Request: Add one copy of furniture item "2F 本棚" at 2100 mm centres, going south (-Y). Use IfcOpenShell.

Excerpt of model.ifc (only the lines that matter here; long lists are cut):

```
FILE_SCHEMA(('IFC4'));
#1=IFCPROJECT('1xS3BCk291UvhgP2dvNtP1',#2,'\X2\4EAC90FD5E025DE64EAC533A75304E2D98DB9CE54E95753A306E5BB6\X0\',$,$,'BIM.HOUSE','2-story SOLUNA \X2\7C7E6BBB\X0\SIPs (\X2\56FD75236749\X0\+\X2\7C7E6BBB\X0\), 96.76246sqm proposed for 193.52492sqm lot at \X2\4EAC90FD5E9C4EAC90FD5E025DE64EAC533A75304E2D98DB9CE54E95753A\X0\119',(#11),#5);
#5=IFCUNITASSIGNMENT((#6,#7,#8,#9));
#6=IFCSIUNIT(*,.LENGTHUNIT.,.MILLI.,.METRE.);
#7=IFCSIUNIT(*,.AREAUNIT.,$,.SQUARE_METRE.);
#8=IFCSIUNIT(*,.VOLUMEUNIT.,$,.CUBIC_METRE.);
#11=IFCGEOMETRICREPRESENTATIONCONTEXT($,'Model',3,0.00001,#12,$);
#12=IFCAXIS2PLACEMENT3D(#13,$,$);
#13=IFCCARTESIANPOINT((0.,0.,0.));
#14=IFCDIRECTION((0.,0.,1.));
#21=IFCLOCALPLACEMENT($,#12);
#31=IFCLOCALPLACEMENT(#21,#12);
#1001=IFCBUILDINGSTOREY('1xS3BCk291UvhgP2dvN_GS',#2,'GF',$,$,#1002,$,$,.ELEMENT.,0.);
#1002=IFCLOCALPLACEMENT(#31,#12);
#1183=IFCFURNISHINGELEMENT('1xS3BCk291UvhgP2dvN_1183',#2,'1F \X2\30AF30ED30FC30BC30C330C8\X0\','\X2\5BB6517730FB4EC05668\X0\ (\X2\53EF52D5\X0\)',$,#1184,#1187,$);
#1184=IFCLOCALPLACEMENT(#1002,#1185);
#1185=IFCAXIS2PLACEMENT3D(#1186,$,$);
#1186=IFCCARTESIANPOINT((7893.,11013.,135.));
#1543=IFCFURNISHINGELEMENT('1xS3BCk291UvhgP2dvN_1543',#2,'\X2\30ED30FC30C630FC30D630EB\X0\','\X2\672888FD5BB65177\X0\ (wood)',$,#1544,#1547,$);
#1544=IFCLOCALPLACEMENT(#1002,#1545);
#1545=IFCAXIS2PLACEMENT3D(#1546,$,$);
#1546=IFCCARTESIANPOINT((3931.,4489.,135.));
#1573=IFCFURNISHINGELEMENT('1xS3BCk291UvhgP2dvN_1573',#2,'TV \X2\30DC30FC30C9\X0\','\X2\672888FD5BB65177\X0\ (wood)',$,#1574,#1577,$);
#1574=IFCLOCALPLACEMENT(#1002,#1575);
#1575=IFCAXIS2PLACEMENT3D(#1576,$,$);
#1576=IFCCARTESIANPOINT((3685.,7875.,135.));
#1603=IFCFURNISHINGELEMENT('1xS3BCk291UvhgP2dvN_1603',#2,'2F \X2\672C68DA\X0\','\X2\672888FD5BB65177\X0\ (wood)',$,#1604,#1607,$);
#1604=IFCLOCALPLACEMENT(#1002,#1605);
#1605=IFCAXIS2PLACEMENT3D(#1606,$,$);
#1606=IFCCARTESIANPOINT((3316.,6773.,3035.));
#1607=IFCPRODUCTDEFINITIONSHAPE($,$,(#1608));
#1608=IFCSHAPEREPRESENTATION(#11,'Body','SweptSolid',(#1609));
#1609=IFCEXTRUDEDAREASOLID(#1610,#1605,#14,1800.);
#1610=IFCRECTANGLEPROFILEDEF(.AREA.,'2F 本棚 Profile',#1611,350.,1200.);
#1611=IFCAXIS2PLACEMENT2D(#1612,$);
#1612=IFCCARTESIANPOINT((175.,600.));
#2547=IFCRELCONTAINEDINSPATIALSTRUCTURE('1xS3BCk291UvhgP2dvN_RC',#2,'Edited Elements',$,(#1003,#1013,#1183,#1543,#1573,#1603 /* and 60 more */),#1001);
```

```python
import numpy as np
import ifcopenshell
import ifcopenshell.api.geometry
import ifcopenshell.api.root
import ifcopenshell.util.element
import ifcopenshell.util.placement
import ifcopenshell.util.unit

model = ifcopenshell.open("model.ifc")
unit_scale = ifcopenshell.util.unit.calculate_unit_scale(model)


def reuse_history(source, copy):
    """copy_class also copies each property set's owner history, people and application; keep the originals."""
    for rel in copy.IsDefinedBy:
        if rel.is_a("IfcRelDefinesByProperties") and (history := rel.RelatingPropertyDefinition.OwnerHistory):
            rel.RelatingPropertyDefinition.OwnerHistory = source.OwnerHistory
            ifcopenshell.util.element.remove_deep2(model, history)


source = model.by_id(1603)
base = ifcopenshell.util.placement.get_local_placement(source.ObjectPlacement)
step = np.array([0.0, -1.0, 0.0]) * 2.1 / unit_scale

for i in range(1, 2):
    copy = ifcopenshell.api.root.copy_class(model, product=source)
    copy.Representation = ifcopenshell.util.element.copy_deep(
        model, source.Representation, exclude=["IfcGeometricRepresentationContext", "IfcRepresentationMap"]
    )
    reuse_history(source, copy)
    matrix = base.copy()
    matrix[:3, 3] += i * step
    print("added at", matrix[:3, 3].round(3) + 0.0)
    ifcopenshell.api.geometry.edit_object_placement(model, product=copy, matrix=matrix, is_si=False)

model.write("model-out.ifc")
```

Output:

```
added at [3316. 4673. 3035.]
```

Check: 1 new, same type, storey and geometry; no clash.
